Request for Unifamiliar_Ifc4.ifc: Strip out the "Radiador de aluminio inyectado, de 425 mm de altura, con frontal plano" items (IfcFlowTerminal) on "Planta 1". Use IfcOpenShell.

First a look at what the model holds.

```python
import ifcopenshell
import ifcopenshell.util.element

model = ifcopenshell.open("Unifamiliar_Ifc4.ifc")
print(model.schema)
storey = next(s for s in model.by_type("IfcBuildingStorey") if s.Name == "Planta 1")
terminals = [e for e in ifcopenshell.util.element.get_decomposition(storey) if e.is_a("IfcFlowTerminal")]
seen = {}
for e in terminals:
    element_type = ifcopenshell.util.element.get_type(e)
    name = element_type.Name if element_type not in (None, e) else None
    seen[name] = seen.get(name, 0) + 1
for name, count in sorted(seen.items(), key=str):
    print(count, "x", name)
```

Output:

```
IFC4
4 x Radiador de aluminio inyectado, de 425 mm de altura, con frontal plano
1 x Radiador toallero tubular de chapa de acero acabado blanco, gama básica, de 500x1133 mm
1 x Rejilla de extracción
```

```python
import ifcopenshell
import ifcopenshell.api.root
import ifcopenshell.util.element

model = ifcopenshell.open("Unifamiliar_Ifc4.ifc")

storey = next(s for s in model.by_type("IfcBuildingStorey") if s.Name == "Planta 1")
terminals = [e for e in ifcopenshell.util.element.get_decomposition(storey) if e.is_a("IfcFlowTerminal")]
targets = [e for e in terminals if (t := ifcopenshell.util.element.get_type(e)) not in (None, e) and t.Name == "Radiador de aluminio inyectado, de 425 mm de altura, con frontal plano"]

for e in targets:
    ifcopenshell.api.root.remove_product(model, product=e)
print(len(targets), "removed")

model.write("Unifamiliar_Ifc4_edited.ifc")
```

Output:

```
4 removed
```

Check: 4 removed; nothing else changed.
